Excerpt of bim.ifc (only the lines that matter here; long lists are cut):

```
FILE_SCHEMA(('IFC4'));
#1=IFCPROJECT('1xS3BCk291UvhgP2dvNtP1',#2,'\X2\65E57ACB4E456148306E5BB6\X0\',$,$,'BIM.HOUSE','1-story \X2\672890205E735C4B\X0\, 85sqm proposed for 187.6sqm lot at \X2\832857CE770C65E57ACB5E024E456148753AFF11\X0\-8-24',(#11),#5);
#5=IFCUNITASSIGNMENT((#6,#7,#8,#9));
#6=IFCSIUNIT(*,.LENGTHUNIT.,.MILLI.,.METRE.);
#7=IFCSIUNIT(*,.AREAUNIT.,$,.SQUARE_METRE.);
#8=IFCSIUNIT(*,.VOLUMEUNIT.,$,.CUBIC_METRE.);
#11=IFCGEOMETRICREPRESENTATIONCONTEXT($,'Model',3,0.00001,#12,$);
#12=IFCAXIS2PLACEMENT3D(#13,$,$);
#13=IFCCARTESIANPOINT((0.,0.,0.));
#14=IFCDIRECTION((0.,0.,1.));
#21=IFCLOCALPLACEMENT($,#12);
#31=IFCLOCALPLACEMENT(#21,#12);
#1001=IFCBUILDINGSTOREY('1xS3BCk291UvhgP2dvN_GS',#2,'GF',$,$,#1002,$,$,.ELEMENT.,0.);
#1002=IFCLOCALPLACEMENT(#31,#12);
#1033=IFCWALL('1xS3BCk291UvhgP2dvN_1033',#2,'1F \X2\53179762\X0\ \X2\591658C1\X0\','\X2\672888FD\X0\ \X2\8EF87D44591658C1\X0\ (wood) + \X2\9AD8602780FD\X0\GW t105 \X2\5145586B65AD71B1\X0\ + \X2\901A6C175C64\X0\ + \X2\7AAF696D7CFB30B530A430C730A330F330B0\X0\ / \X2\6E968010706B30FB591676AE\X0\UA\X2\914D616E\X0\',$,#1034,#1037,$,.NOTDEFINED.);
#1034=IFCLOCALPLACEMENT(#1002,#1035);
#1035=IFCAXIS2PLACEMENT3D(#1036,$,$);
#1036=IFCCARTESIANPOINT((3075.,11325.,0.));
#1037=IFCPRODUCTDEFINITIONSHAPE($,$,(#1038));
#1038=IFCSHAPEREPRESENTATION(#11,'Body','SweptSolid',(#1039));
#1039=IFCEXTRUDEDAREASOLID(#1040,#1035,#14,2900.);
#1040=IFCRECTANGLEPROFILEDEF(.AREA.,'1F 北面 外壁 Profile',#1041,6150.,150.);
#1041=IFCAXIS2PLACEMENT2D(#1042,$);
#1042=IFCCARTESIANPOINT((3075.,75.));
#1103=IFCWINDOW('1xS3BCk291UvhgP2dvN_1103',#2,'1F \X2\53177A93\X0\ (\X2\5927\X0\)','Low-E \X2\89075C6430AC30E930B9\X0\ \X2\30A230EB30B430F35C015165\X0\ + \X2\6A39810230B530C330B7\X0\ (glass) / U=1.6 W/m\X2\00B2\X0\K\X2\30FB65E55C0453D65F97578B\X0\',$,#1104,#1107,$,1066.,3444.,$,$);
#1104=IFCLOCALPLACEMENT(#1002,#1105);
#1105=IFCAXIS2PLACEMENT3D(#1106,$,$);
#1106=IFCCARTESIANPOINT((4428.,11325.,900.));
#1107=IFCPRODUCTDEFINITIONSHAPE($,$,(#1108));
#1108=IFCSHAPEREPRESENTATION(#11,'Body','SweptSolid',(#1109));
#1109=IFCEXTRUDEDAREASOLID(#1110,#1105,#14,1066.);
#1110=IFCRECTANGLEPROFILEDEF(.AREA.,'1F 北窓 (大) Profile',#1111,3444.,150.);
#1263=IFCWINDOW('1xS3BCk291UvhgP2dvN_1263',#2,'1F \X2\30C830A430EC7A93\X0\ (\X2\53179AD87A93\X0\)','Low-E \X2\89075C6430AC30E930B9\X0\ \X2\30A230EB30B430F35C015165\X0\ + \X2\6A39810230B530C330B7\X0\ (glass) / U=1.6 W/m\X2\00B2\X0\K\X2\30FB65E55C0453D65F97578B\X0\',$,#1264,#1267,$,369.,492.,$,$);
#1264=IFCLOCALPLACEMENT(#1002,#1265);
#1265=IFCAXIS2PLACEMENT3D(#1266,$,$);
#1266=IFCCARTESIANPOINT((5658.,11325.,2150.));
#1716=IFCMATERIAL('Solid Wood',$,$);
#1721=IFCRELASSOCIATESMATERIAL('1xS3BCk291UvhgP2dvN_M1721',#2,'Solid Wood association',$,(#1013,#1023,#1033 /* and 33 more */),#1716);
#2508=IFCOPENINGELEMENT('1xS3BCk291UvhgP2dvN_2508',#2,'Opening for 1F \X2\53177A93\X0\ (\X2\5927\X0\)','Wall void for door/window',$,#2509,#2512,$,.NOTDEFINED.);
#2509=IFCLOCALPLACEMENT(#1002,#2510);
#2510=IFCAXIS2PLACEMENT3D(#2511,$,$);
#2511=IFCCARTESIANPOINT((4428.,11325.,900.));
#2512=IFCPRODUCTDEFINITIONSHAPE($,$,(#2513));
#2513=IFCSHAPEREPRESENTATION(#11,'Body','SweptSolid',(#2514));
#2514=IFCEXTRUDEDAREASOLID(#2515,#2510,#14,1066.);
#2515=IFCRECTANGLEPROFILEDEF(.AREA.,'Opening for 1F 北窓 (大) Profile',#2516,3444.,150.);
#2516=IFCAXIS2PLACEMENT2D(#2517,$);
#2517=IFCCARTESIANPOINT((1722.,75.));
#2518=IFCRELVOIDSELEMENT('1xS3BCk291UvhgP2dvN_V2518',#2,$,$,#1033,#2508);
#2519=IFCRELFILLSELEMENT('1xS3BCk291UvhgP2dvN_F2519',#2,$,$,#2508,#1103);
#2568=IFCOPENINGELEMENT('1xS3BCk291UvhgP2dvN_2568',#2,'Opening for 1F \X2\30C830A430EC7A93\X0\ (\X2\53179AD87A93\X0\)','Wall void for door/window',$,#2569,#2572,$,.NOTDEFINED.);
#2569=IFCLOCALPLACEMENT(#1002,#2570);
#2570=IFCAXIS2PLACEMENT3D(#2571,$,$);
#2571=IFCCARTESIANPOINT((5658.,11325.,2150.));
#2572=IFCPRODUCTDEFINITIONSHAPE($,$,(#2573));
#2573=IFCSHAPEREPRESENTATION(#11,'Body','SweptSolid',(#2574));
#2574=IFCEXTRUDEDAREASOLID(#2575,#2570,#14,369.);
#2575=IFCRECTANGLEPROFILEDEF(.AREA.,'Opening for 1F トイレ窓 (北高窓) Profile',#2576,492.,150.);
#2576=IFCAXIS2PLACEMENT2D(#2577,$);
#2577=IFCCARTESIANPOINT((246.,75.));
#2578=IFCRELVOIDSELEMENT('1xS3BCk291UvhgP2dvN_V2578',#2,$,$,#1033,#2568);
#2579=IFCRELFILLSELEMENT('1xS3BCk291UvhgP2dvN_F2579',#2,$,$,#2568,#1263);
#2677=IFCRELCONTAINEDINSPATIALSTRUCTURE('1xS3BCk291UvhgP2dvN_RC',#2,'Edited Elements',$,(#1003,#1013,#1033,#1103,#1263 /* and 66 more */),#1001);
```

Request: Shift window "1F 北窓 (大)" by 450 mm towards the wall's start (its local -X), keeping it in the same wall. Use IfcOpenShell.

```python
import ifcopenshell
import ifcopenshell.api.geometry
import ifcopenshell.util.placement
import ifcopenshell.util.unit

model = ifcopenshell.open("bim.ifc")
unit_scale = ifcopenshell.util.unit.calculate_unit_scale(model)

window = model.by_guid("1xS3BCk291UvhgP2dvN_1103")
opening = window.FillsVoids[0].RelatingOpeningElement
wall = opening.VoidsElements[0].RelatingBuildingElement

wall_matrix = ifcopenshell.util.placement.get_local_placement(wall.ObjectPlacement)
shift = wall_matrix[:3, 0] * -0.45 / unit_scale
before = ifcopenshell.util.placement.get_local_placement(window.ObjectPlacement)[:3, 3].copy()

# The window is not placed relative to its opening, so move both.
for product in (opening, window):
    matrix = ifcopenshell.util.placement.get_local_placement(product.ObjectPlacement)
    matrix[:3, 3] += shift
    ifcopenshell.api.geometry.edit_object_placement(model, product=product, matrix=matrix, is_si=False)

after = ifcopenshell.util.placement.get_local_placement(window.ObjectPlacement)[:3, 3]
print("window moved by", (after - before).round(3) + 0.0)

model.write("bim_edited.ifc")
```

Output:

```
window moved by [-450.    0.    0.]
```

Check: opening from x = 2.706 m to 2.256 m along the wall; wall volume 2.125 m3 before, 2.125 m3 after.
